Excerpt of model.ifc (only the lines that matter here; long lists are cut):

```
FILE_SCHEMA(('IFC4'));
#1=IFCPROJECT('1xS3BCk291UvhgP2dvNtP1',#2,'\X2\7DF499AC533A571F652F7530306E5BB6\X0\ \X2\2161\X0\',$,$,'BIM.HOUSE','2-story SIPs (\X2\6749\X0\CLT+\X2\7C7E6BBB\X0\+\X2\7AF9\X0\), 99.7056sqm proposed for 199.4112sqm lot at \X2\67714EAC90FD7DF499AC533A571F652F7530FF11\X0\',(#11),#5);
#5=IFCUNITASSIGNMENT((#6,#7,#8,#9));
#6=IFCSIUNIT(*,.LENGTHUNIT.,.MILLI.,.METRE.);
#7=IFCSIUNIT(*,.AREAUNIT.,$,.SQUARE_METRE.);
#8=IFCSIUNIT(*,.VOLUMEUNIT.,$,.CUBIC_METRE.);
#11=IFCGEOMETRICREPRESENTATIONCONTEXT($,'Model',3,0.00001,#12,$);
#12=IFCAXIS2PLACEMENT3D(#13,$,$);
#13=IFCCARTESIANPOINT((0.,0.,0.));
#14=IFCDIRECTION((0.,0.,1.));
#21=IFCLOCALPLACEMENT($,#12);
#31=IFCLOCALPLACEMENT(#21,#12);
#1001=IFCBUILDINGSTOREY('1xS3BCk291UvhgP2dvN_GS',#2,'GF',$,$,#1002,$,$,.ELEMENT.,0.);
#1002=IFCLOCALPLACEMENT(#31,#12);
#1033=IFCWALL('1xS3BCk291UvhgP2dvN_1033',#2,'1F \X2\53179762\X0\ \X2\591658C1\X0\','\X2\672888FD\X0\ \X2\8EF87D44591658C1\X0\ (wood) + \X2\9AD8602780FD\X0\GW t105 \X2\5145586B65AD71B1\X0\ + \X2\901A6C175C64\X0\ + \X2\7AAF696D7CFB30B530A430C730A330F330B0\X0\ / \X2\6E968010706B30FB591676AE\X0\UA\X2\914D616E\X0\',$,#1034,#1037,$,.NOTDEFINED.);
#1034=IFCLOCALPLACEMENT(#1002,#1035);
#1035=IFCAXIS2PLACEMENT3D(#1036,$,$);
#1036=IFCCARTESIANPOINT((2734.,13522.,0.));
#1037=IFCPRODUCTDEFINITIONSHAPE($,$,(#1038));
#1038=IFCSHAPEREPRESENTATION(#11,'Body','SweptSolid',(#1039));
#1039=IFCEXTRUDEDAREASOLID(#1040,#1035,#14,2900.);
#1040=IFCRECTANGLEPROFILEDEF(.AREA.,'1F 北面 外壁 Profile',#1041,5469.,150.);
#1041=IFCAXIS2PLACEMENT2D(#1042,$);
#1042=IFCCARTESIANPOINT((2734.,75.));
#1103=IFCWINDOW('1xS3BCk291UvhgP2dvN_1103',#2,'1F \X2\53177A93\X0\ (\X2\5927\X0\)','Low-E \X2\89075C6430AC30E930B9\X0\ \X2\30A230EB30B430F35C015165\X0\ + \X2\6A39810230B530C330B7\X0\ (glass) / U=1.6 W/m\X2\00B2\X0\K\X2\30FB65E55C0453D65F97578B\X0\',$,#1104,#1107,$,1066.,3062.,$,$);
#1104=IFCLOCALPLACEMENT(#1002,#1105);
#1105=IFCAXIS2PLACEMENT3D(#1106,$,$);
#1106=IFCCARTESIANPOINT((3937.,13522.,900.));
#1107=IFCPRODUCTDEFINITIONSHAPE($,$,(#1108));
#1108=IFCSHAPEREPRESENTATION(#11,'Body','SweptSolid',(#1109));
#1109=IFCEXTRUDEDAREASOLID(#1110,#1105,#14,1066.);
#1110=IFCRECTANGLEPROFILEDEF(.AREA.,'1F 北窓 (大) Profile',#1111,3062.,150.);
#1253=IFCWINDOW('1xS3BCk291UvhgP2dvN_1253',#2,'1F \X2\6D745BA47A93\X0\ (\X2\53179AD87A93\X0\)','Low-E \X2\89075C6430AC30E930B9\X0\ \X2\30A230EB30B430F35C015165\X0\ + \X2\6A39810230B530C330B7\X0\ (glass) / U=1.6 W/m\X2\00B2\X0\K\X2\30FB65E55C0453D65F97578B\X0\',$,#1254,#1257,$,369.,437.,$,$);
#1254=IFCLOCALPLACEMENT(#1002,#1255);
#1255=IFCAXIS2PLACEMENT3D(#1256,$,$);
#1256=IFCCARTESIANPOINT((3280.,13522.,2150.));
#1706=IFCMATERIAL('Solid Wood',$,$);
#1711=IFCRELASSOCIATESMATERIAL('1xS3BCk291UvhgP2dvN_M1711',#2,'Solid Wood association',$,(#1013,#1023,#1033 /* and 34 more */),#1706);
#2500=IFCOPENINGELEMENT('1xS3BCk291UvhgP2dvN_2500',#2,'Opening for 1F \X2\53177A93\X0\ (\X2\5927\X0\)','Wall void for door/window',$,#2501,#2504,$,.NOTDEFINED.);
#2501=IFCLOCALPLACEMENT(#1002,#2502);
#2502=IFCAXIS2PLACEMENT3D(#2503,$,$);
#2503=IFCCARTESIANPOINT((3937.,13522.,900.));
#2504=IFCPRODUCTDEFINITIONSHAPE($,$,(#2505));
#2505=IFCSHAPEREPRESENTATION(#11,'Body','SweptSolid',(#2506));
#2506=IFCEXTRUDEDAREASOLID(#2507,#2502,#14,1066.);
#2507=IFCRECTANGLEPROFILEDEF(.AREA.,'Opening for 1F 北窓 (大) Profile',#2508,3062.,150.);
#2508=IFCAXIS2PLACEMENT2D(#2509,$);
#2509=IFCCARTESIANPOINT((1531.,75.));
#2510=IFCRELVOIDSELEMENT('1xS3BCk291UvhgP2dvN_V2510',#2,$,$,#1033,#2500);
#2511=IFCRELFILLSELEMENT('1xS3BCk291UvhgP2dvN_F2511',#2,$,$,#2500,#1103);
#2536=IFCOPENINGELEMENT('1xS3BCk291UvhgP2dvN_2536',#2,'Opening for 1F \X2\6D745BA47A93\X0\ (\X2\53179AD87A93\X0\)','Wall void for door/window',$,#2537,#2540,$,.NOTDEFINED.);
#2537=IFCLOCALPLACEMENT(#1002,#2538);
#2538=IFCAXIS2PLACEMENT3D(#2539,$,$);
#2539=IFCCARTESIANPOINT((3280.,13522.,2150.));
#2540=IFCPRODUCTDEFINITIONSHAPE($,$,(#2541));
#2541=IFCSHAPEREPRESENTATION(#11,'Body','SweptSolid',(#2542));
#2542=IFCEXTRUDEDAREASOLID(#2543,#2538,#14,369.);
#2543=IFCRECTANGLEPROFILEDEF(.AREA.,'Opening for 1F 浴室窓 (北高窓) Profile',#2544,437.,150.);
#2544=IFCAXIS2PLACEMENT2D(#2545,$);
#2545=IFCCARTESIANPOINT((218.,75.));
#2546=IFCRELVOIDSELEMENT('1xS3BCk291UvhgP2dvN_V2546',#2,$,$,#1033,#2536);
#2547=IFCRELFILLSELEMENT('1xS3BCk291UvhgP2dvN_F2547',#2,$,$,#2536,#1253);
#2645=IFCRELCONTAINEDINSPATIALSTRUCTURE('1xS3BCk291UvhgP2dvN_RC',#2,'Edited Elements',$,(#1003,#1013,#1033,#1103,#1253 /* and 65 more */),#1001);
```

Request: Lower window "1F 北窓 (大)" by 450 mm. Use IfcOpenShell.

```python
import numpy as np
import ifcopenshell
import ifcopenshell.api.geometry
import ifcopenshell.util.placement
import ifcopenshell.util.unit

model = ifcopenshell.open("model.ifc")
unit_scale = ifcopenshell.util.unit.calculate_unit_scale(model)

window = model.by_id(1103)
opening = window.FillsVoids[0].RelatingOpeningElement
dz = -450.0

shift = np.array([0.0, 0.0, dz])
# The window is not placed relative to its opening, so move both.
for product in (opening, window):
    matrix = ifcopenshell.util.placement.get_local_placement(product.ObjectPlacement)
    matrix[:3, 3] += shift
    ifcopenshell.api.geometry.edit_object_placement(model, product=product, matrix=matrix, is_si=False)

print(f"moved by {dz * unit_scale:+.3f} m")

model.write("model_updated.ifc")
```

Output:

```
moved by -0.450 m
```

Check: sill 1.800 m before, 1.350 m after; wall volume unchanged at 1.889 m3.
